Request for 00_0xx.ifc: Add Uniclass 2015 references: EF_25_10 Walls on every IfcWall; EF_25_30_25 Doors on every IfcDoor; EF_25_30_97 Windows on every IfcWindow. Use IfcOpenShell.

First a look at what the model holds.

```python
import ifcopenshell

model = ifcopenshell.open("00_0xx.ifc")
print(model.schema)
print("classifications:", [c.Name for c in model.by_type("IfcClassification")])
for ifc_class in ("IfcDoor", "IfcRoof", "IfcStair", "IfcWall", "IfcWindow"):
    print(ifc_class, len(model.by_type(ifc_class)))
```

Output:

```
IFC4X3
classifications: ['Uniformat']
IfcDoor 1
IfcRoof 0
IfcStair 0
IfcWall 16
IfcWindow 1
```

```python
import ifcopenshell
import ifcopenshell.api.classification

model = ifcopenshell.open("00_0xx.ifc")

system = ifcopenshell.api.classification.add_classification(model, classification="Uniclass 2015")

codes = {
    "IfcWall": ("EF_25_10", "Walls"),
    "IfcDoor": ("EF_25_30_25", "Doors"),
    "IfcWindow": ("EF_25_30_97", "Windows"),
}
for ifc_class, (code, name) in codes.items():
    products = model.by_type(ifc_class)
    ifcopenshell.api.classification.add_reference(
        model, products=products, classification=system, identification=code, name=name
    )
    print(code, len(products))

model.write("00_0xx_v2.ifc")
```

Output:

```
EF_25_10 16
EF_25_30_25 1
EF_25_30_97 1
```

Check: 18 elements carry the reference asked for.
